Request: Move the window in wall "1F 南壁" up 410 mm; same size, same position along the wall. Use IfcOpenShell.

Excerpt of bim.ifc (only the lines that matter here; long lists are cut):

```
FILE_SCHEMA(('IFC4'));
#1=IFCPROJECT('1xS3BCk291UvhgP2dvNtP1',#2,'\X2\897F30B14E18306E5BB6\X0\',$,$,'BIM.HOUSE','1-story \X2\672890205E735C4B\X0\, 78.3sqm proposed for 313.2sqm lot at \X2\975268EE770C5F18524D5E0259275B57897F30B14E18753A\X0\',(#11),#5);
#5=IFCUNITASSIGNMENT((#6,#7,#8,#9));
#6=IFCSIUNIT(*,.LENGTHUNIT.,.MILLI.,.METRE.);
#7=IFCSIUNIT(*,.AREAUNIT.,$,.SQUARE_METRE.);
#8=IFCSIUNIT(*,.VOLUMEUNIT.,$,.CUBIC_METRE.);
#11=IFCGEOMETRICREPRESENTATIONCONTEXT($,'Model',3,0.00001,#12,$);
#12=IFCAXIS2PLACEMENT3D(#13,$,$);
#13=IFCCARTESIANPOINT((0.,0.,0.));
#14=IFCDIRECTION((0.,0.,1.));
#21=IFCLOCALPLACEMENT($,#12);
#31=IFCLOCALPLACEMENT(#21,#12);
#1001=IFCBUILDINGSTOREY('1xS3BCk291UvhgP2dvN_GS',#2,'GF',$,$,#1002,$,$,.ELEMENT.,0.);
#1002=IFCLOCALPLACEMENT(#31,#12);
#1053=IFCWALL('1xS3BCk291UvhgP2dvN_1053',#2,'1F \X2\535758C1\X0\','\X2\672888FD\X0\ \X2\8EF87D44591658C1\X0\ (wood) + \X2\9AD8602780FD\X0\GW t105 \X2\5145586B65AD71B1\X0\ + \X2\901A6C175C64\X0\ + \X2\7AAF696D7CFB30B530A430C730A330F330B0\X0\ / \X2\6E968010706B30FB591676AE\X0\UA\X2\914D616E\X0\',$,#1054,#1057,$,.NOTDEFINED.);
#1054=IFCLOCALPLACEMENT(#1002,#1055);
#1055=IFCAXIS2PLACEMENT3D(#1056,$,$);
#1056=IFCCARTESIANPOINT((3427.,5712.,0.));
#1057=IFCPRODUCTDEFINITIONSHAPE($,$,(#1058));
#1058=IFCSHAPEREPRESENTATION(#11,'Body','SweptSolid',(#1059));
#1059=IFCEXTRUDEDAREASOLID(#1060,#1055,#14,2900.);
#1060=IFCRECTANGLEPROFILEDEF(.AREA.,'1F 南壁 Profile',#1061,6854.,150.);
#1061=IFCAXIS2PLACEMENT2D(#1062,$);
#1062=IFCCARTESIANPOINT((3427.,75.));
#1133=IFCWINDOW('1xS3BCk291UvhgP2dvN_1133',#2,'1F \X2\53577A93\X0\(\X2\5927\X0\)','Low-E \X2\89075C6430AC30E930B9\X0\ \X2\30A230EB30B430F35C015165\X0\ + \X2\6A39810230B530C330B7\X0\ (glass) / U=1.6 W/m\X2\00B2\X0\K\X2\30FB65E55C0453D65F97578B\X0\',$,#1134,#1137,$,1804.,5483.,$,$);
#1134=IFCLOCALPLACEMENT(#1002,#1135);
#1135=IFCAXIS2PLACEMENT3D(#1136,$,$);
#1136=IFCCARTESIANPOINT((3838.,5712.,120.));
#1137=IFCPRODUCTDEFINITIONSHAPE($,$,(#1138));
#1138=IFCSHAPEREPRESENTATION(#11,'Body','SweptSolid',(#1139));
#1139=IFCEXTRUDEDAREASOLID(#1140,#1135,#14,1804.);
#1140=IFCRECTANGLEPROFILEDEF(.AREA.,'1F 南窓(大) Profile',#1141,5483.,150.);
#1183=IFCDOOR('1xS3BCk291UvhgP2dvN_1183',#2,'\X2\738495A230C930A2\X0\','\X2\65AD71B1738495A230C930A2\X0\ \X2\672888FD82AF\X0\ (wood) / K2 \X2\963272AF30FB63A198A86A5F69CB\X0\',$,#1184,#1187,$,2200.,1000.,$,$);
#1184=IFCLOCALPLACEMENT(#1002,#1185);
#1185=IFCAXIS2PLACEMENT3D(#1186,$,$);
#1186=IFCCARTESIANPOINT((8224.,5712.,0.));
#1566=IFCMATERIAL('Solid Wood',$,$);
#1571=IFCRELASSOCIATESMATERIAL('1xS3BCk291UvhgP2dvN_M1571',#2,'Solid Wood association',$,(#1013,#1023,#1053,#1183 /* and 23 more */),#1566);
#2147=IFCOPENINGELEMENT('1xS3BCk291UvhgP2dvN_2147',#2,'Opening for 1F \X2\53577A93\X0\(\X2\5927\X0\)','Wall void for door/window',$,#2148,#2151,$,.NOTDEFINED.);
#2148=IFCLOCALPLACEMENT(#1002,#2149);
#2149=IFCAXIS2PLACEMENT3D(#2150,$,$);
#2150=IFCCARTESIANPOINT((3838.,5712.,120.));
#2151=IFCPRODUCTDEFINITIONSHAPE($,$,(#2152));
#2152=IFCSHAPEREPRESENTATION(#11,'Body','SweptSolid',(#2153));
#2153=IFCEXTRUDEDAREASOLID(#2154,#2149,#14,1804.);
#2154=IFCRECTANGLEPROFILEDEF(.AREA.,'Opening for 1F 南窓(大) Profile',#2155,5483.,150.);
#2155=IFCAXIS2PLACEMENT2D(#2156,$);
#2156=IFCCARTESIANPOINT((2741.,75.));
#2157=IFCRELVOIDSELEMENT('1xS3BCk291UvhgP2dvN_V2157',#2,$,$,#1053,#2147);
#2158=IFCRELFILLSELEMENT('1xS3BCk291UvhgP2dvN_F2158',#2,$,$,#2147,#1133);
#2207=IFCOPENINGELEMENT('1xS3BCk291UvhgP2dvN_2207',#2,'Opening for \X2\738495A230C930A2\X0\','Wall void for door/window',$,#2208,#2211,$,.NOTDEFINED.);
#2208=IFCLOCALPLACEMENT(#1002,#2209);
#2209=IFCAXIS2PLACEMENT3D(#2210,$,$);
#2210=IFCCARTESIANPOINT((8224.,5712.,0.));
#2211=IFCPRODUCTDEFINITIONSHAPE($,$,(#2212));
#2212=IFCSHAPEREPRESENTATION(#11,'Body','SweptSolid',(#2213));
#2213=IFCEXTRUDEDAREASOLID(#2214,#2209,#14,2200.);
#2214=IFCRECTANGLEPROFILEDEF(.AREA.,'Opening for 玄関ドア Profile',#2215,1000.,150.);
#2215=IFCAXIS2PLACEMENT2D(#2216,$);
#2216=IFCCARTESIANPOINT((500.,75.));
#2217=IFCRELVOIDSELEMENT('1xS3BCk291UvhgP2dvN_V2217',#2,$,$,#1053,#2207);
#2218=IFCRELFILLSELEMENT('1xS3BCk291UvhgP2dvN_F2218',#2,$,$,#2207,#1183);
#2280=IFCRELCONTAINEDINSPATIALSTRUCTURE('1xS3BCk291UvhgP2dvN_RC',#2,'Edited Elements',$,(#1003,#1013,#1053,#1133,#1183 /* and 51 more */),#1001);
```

```python
import numpy as np
import ifcopenshell
import ifcopenshell.api.geometry
import ifcopenshell.util.placement
import ifcopenshell.util.unit

model = ifcopenshell.open("bim.ifc")
unit_scale = ifcopenshell.util.unit.calculate_unit_scale(model)

window = model.by_guid("1xS3BCk291UvhgP2dvN_1133")
opening = window.FillsVoids[0].RelatingOpeningElement
dz = 410.0

shift = np.array([0.0, 0.0, dz])
# The window is not placed relative to its opening, so move both.
for product in (opening, window):
    matrix = ifcopenshell.util.placement.get_local_placement(product.ObjectPlacement)
    matrix[:3, 3] += shift
    ifcopenshell.api.geometry.edit_object_placement(model, product=product, matrix=matrix, is_si=False)

print(f"moved by {dz * unit_scale:+.3f} m")

model.write("bim_updated.ifc")
```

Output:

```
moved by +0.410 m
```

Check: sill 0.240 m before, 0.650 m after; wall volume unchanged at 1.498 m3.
